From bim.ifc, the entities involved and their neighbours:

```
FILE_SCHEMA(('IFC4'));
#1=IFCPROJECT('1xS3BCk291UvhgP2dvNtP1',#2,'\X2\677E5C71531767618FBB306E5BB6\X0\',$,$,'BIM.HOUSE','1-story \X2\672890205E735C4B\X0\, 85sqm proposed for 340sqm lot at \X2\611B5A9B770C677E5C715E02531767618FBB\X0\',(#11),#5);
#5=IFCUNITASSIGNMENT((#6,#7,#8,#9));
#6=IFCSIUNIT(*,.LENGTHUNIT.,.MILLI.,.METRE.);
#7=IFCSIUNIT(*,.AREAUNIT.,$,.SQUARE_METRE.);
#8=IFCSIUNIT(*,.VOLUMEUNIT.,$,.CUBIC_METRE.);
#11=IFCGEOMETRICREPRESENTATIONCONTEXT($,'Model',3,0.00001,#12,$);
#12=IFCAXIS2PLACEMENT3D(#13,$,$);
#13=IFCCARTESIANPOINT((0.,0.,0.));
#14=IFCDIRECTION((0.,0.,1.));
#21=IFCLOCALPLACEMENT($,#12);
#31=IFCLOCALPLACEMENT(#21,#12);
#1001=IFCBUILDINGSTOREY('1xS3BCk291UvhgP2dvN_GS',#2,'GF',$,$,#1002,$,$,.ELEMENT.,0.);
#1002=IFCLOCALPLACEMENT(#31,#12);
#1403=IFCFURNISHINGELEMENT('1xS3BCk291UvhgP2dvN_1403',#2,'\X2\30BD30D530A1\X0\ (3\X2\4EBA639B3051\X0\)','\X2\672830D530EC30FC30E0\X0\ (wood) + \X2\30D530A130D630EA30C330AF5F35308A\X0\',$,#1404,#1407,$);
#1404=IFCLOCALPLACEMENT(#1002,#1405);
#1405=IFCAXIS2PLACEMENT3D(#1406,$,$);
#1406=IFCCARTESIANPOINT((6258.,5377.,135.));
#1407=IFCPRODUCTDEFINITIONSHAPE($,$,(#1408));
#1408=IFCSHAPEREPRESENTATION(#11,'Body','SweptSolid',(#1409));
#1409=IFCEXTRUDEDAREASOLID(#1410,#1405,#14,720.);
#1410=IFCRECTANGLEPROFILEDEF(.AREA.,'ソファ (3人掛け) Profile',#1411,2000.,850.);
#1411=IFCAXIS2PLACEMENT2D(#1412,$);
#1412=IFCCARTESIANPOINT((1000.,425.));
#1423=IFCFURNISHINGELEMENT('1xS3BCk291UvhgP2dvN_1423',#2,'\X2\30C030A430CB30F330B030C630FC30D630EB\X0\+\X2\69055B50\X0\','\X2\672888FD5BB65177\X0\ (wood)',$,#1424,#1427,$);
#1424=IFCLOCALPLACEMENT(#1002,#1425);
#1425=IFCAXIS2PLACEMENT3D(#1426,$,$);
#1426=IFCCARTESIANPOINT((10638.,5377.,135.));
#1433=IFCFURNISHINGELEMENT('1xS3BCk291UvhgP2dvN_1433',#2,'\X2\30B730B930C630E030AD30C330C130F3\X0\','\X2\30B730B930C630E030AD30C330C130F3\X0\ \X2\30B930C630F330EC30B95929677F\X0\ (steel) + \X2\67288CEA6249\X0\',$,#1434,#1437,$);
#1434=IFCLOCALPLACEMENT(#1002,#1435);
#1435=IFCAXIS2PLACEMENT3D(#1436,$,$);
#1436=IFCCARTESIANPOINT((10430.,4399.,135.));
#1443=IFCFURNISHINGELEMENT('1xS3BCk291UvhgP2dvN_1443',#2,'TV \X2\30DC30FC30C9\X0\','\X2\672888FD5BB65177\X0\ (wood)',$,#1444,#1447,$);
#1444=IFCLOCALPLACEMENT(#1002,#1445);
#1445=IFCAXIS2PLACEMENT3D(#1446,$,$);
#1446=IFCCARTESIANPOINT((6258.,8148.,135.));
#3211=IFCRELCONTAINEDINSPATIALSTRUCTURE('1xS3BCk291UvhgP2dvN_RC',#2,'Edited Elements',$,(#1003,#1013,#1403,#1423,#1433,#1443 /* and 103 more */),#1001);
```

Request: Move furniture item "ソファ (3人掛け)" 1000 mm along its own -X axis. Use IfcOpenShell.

```python
import ifcopenshell
import ifcopenshell.api.geometry
import ifcopenshell.util.placement
import ifcopenshell.util.unit

model = ifcopenshell.open("bim.ifc")
unit_scale = ifcopenshell.util.unit.calculate_unit_scale(model)

item = model.by_guid("1xS3BCk291UvhgP2dvN_1403")
matrix = ifcopenshell.util.placement.get_local_placement(item.ObjectPlacement)
matrix[:3, 3] -= matrix[:3, 0] * 1 / unit_scale
ifcopenshell.api.geometry.edit_object_placement(model, product=item, matrix=matrix, is_si=False)

print(ifcopenshell.util.placement.get_local_placement(item.ObjectPlacement).round(3) + 0.0)

model.write("bim-out.ifc")
```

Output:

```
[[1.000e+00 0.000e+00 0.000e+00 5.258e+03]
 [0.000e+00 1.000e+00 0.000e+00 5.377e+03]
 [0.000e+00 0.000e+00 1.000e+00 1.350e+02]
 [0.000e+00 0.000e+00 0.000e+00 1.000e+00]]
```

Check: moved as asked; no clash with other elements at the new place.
